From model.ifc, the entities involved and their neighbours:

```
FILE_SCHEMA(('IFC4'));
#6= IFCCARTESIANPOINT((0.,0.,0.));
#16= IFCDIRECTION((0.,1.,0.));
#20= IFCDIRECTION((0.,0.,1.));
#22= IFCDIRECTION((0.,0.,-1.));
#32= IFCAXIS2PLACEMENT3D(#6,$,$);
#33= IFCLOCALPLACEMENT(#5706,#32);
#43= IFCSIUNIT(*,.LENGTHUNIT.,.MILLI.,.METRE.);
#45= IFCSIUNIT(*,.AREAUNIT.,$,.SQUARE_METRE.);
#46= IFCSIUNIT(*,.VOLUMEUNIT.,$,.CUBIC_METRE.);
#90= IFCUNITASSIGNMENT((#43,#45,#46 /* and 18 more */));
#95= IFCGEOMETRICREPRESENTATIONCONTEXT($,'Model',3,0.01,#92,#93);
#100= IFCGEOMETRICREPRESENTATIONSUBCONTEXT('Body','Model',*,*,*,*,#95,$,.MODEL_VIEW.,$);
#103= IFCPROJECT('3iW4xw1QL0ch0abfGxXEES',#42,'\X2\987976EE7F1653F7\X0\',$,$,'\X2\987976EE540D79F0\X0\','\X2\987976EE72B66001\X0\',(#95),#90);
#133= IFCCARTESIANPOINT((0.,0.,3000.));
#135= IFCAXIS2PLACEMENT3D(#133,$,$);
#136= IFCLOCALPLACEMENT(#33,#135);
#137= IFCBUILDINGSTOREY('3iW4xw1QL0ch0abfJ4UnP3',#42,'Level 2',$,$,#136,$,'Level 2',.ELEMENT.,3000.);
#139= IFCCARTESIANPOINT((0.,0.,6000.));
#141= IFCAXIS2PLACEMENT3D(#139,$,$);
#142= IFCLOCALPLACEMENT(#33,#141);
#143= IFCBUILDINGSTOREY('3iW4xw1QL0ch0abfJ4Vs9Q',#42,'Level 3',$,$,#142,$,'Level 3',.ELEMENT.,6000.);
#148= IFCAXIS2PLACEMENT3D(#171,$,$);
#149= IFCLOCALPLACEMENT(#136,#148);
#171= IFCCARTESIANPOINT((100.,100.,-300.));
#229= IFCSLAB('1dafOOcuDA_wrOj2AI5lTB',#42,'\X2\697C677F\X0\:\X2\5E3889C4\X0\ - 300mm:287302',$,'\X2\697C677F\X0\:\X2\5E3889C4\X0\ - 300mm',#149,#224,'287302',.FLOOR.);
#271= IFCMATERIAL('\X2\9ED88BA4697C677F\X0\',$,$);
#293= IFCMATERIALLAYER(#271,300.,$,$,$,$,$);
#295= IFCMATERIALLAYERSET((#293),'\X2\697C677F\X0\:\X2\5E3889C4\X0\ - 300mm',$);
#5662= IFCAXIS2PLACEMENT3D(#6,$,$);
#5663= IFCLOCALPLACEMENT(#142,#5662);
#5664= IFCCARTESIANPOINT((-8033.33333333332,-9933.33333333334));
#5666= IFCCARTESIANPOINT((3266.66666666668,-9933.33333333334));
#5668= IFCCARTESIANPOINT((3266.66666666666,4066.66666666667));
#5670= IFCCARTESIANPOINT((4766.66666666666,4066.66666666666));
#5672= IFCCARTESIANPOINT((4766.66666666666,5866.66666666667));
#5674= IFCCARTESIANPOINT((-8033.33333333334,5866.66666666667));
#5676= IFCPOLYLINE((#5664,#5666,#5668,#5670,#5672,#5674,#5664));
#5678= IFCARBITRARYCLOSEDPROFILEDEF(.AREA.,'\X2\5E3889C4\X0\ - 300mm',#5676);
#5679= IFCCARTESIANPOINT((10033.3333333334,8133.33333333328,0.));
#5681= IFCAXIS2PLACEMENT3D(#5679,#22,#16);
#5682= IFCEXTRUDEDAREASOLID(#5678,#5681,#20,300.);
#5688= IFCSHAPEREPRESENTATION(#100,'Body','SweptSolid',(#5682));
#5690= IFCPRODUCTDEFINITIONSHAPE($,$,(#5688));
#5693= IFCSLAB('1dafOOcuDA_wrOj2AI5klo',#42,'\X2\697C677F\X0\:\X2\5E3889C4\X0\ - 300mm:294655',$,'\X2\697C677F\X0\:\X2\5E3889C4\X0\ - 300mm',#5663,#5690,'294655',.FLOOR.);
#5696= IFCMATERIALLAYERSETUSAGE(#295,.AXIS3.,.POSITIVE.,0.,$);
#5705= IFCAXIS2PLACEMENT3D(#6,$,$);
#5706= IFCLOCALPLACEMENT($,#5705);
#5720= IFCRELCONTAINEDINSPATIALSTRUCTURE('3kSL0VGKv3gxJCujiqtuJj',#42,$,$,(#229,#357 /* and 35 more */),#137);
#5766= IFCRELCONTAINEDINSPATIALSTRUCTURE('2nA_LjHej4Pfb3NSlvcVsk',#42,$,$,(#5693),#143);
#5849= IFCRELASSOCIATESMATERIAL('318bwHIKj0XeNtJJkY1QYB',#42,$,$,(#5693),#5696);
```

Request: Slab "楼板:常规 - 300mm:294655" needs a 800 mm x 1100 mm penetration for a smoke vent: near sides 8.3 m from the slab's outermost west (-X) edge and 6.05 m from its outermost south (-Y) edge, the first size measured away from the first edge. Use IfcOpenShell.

```python
import numpy as np
import ifcopenshell
import ifcopenshell.api.feature
import ifcopenshell.api.geometry
import ifcopenshell.api.root
import ifcopenshell.geom
import ifcopenshell.util.placement
import ifcopenshell.util.representation
import ifcopenshell.util.shape
import ifcopenshell.util.unit

model = ifcopenshell.open("model.ifc")
unit_scale = ifcopenshell.util.unit.calculate_unit_scale(model)
settings = ifcopenshell.geom.settings()


def volume(element):
    """Net volume in cubic metres, openings subtracted."""
    shape = ifcopenshell.geom.create_shape(settings, element)
    return ifcopenshell.util.shape.get_volume(shape.geometry)


slab = model.by_guid("1dafOOcuDA_wrOj2AI5klo")
before = volume(slab)

# Extent in the slab's own axes, in metres. The edges named are its -X and -Y sides.
slab_shape = ifcopenshell.geom.create_shape(settings, slab)
vertices = ifcopenshell.util.shape.get_vertices(slab_shape.geometry)
x_min, y_min, bottom = vertices.min(axis=0)
top = vertices[:, 2].max()

opening = ifcopenshell.api.root.create_entity(model, ifc_class="IfcOpeningElement", name="Smoke vent opening", predefined_type="OPENING")
context = ifcopenshell.util.representation.get_context(model, "Model", "Body", "MODEL_VIEW")
width, depth = 0.8, 1.1
outline = [(0.0, 0.0), (width, 0.0), (width, depth), (0.0, depth), (0.0, 0.0)]
# Overshoot both faces by 50 mm so the cut is clean.
shape = ifcopenshell.api.geometry.add_slab_representation(
    model, context=context, depth=top - bottom + 0.1, polyline=outline
)
ifcopenshell.api.geometry.assign_representation(model, product=opening, representation=shape)

matrix = ifcopenshell.util.placement.get_local_placement(slab.ObjectPlacement)
matrix[:, 3] = matrix @ np.append(np.array([x_min + 8.3, y_min + 6.05, bottom - 0.05]) / unit_scale, 1.0)
ifcopenshell.api.geometry.edit_object_placement(model, product=opening, matrix=matrix, is_si=False)
ifcopenshell.api.feature.add_feature(model, feature=opening, element=slab)

after = volume(slab)

print(f"slab volume {before:.3f} -> {after:.3f} m3")

model.write("model_v2.ifc")
```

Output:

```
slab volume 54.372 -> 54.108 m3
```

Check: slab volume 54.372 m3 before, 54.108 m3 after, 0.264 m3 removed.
